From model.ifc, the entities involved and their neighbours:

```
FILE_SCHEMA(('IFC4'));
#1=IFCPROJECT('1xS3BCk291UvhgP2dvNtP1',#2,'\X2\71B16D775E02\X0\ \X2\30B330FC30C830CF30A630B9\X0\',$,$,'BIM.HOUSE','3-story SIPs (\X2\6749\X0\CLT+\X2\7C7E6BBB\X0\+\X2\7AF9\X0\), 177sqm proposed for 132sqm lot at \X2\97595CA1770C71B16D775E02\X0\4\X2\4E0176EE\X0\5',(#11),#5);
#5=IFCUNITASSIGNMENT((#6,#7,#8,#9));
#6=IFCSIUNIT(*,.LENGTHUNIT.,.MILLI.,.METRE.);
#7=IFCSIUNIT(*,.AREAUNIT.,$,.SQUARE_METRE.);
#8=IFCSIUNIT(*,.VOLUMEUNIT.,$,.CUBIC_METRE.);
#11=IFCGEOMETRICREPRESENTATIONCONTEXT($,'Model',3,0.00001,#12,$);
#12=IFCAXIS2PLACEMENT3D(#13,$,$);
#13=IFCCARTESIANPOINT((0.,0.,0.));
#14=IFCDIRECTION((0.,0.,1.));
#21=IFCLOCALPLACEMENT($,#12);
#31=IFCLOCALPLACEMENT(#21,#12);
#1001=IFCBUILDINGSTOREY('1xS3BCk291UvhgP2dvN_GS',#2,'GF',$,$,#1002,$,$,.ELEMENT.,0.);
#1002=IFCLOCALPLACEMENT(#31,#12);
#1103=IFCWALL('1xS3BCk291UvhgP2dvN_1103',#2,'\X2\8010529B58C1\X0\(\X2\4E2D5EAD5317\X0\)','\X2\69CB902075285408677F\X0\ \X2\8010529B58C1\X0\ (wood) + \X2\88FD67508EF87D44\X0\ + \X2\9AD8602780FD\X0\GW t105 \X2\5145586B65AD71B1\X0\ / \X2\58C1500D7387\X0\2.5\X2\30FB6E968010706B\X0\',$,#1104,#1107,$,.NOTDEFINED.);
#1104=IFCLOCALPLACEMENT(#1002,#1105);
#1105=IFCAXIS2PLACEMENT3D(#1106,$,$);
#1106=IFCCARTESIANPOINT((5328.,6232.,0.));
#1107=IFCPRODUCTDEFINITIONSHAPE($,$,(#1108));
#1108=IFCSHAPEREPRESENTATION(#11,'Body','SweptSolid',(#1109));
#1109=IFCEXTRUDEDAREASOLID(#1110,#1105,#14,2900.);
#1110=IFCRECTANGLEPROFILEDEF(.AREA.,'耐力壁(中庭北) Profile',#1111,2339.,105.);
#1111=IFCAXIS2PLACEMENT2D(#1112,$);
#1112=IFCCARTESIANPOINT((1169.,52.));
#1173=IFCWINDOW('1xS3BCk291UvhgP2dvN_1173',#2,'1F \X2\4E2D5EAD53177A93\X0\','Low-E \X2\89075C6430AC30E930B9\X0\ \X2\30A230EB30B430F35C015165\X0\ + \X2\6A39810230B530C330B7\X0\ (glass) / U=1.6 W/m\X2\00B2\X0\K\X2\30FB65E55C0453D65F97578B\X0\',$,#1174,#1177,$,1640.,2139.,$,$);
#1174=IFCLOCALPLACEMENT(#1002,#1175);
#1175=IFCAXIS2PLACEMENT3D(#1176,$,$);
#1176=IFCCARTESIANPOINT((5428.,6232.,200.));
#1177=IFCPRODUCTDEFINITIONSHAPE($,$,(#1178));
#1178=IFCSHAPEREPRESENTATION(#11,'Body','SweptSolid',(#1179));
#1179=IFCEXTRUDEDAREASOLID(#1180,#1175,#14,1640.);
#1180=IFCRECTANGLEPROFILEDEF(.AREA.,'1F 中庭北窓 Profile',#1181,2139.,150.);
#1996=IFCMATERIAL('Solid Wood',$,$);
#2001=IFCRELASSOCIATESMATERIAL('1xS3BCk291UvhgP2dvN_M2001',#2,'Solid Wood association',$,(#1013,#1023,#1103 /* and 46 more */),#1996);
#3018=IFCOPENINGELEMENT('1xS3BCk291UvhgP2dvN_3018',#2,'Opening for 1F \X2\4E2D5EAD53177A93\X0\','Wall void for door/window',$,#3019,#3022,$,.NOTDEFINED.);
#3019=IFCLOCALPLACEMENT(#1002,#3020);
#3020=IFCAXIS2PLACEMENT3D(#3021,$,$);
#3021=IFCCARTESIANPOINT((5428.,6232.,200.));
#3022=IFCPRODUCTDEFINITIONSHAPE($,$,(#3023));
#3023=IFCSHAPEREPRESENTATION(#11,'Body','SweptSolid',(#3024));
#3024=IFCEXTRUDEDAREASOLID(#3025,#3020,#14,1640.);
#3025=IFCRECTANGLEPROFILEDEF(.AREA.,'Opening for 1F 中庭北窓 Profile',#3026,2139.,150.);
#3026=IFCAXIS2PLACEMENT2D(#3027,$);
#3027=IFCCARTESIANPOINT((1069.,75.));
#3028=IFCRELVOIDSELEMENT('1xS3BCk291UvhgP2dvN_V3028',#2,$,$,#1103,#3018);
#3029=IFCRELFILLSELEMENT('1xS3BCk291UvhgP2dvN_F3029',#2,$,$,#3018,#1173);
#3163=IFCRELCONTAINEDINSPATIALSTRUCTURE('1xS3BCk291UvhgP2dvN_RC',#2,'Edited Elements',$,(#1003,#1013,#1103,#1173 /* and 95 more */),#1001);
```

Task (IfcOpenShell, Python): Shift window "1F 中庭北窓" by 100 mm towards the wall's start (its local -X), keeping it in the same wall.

```python
import ifcopenshell
import ifcopenshell.api.geometry
import ifcopenshell.util.placement

model = ifcopenshell.open("model.ifc")

window = model.by_guid("1xS3BCk291UvhgP2dvN_1173")
opening = window.FillsVoids[0].RelatingOpeningElement
wall = opening.VoidsElements[0].RelatingBuildingElement

wall_matrix = ifcopenshell.util.placement.get_local_placement(wall.ObjectPlacement)
shift = wall_matrix[:3, 0] * -100.0
before = ifcopenshell.util.placement.get_local_placement(window.ObjectPlacement)[:3, 3].copy()

# The window is not placed relative to its opening, so move both.
for product in (opening, window):
    matrix = ifcopenshell.util.placement.get_local_placement(product.ObjectPlacement)
    matrix[:3, 3] += shift
    ifcopenshell.api.geometry.edit_object_placement(model, product=product, matrix=matrix, is_si=False)

after = ifcopenshell.util.placement.get_local_placement(window.ObjectPlacement)[:3, 3]
print("window moved by", (after - before).round(3) + 0.0)

model.write("model-out.ifc")
```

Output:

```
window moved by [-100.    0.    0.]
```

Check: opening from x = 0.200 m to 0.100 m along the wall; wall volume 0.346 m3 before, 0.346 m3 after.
